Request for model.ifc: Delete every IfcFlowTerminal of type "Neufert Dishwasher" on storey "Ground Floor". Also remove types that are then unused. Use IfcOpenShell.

First a look at what the model holds.

```python
import ifcopenshell
import ifcopenshell.util.element

model = ifcopenshell.open("model.ifc")
print(model.schema)
storey = next(s for s in model.by_type("IfcBuildingStorey") if s.Name == "Ground Floor")
terminals = [e for e in ifcopenshell.util.element.get_decomposition(storey) if e.is_a("IfcFlowTerminal")]
seen = {}
for e in terminals:
    element_type = ifcopenshell.util.element.get_type(e)
    name = element_type.Name if element_type not in (None, e) else None
    seen[name] = seen.get(name, 0) + 1
for name, count in sorted(seen.items(), key=str):
    print(count, "x", name)
```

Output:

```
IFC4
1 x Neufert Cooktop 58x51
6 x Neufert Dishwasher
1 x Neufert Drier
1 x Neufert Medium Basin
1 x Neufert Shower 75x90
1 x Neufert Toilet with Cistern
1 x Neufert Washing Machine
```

```python
import ifcopenshell
import ifcopenshell.api.root
import ifcopenshell.util.element

model = ifcopenshell.open("model.ifc")

storey = next(s for s in model.by_type("IfcBuildingStorey") if s.Name == "Ground Floor")
terminals = [e for e in ifcopenshell.util.element.get_decomposition(storey) if e.is_a("IfcFlowTerminal")]
targets = [e for e in terminals if (t := ifcopenshell.util.element.get_type(e)) not in (None, e) and t.Name == "Neufert Dishwasher"]
types = {ifcopenshell.util.element.get_type(e) for e in targets} - {None, *targets}

for e in targets:
    ifcopenshell.api.root.remove_product(model, product=e)
print(len(targets), "removed")

unused = [t for t in types if not ifcopenshell.util.element.get_types(t)]
for t in unused:
    ifcopenshell.api.root.remove_product(model, product=t)
print(len(unused), "unused types removed")

model.write("model_rev.ifc")
```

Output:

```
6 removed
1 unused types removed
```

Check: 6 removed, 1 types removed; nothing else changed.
